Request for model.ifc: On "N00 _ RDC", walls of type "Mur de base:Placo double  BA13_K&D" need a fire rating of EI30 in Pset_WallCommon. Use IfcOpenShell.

First a look at what the model holds.

```python
import ifcopenshell
import ifcopenshell.util.element

model = ifcopenshell.open("model.ifc")
print(model.schema)
storey = next(s for s in model.by_type("IfcBuildingStorey") if s.Name == "N00 _ RDC")
walls = [e for e in ifcopenshell.util.element.get_decomposition(storey) if e.is_a("IfcWall")]
seen = {}
for e in walls:
    element_type = ifcopenshell.util.element.get_type(e)
    key = (element_type.Name if element_type != e and element_type else None, ifcopenshell.util.element.get_pset(e, "Pset_WallCommon", "FireRating"))
    seen[key] = seen.get(key, 0) + 1
for (name, value), count in sorted(seen.items(), key=str):
    print(count, "x", name, "|", value)
```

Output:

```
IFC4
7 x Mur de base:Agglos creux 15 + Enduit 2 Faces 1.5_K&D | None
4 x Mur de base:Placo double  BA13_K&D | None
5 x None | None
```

```python
import ifcopenshell
import ifcopenshell.api.pset
import ifcopenshell.util.element

model = ifcopenshell.open("model.ifc")

storey = next(s for s in model.by_type("IfcBuildingStorey") if s.Name == "N00 _ RDC")
walls = [e for e in ifcopenshell.util.element.get_decomposition(storey) if e.is_a("IfcWall")]

count = 0
for e in walls:
    element_type = ifcopenshell.util.element.get_type(e)
    if element_type in (None, e) or element_type.Name != "Mur de base:Placo double  BA13_K&D":
        continue
    # add_pset returns the element's existing set when there is one.
    pset = ifcopenshell.api.pset.add_pset(model, product=e, name="Pset_WallCommon")
    ifcopenshell.api.pset.edit_pset(model, pset=pset, properties={"FireRating": "EI30"})
    count += 1

print(count, "walls updated")

model.write("model_rev.ifc")
```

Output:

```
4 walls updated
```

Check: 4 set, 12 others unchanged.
